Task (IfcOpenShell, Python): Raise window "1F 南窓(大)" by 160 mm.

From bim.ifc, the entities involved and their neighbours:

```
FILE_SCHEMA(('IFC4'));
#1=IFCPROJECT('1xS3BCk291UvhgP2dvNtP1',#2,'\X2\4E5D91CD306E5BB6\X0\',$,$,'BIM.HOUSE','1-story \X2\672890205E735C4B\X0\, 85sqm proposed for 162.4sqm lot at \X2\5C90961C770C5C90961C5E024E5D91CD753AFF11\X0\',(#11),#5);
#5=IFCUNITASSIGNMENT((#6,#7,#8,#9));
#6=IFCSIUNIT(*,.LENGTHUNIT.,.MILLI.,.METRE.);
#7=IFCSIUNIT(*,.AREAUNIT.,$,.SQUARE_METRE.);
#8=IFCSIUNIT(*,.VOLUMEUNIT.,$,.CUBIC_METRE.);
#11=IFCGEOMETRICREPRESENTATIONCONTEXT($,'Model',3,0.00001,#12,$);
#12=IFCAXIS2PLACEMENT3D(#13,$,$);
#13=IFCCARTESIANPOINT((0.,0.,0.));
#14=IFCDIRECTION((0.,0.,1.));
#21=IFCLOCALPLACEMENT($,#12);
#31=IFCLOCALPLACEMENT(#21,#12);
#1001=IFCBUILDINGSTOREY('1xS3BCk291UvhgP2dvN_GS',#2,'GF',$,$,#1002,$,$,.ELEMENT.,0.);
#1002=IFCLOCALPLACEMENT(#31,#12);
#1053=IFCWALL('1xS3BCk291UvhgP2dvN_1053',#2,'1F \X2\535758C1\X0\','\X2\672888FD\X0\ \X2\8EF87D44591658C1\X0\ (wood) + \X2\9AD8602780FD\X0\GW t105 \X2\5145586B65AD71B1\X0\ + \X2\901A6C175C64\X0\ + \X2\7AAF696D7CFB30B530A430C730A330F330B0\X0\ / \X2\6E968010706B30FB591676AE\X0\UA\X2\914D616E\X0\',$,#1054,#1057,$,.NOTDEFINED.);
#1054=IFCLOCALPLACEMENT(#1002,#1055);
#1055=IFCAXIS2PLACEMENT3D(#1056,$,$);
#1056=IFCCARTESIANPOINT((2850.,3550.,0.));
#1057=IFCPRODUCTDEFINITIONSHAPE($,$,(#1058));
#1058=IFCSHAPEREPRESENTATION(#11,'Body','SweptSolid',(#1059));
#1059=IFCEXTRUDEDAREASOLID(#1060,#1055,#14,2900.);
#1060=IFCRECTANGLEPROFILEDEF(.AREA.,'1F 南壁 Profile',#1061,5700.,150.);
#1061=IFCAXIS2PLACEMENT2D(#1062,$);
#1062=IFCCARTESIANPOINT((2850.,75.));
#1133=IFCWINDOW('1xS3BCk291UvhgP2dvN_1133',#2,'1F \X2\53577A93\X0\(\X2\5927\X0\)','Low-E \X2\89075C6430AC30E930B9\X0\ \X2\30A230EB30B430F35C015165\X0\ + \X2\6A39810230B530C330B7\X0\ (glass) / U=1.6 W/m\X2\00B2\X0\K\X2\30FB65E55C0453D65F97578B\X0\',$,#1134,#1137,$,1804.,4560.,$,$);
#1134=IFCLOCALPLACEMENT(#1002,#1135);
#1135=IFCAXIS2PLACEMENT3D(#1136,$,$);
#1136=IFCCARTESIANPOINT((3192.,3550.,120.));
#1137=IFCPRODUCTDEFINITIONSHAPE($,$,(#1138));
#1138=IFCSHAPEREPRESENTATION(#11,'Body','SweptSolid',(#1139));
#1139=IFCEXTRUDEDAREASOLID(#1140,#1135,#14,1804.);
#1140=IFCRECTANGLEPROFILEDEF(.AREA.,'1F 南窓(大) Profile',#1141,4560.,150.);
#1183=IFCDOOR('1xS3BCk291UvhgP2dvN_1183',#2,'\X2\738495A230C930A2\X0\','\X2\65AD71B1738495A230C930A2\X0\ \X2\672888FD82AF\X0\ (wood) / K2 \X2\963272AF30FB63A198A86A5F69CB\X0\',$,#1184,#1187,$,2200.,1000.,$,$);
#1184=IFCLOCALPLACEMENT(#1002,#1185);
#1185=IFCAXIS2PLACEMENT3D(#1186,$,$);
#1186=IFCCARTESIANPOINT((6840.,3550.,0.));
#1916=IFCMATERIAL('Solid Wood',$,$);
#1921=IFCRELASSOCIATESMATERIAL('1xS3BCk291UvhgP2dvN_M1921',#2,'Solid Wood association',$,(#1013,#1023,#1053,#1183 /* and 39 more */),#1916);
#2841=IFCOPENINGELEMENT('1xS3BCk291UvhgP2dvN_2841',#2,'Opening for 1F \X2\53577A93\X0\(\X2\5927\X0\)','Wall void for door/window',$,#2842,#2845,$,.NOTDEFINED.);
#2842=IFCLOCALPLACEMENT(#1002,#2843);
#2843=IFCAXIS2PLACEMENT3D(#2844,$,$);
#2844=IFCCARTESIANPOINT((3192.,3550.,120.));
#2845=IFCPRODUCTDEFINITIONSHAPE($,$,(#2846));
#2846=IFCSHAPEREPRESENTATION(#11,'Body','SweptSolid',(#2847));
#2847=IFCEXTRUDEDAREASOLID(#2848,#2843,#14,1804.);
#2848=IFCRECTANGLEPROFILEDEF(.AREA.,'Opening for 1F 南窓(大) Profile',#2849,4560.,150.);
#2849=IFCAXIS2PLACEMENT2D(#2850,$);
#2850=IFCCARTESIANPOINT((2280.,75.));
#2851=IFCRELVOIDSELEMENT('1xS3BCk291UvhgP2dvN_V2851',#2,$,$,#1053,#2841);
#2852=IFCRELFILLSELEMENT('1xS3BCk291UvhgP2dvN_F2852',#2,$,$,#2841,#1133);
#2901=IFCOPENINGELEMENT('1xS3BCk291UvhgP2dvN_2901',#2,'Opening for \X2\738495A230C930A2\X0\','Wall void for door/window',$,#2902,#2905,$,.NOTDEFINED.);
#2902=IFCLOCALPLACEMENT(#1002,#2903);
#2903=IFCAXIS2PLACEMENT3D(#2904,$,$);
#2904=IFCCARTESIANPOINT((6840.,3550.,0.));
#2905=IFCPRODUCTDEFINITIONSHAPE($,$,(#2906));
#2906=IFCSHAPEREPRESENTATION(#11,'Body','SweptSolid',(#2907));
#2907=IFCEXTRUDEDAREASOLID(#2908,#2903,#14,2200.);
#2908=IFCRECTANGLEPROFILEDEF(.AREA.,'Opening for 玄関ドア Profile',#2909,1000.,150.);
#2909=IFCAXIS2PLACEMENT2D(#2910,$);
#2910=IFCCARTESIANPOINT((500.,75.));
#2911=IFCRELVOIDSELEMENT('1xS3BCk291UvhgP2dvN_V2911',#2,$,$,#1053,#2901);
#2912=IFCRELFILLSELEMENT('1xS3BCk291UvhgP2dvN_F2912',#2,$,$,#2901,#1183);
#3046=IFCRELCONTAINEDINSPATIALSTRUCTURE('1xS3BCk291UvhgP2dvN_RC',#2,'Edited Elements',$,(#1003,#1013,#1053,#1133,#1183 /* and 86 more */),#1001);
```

```python
import numpy as np
import ifcopenshell
import ifcopenshell.api.geometry
import ifcopenshell.util.placement
import ifcopenshell.util.unit

model = ifcopenshell.open("bim.ifc")
unit_scale = ifcopenshell.util.unit.calculate_unit_scale(model)

window = model.by_guid("1xS3BCk291UvhgP2dvN_1133")
opening = window.FillsVoids[0].RelatingOpeningElement
dz = 160.0

shift = np.array([0.0, 0.0, dz])
# The window is not placed relative to its opening, so move both.
for product in (opening, window):
    matrix = ifcopenshell.util.placement.get_local_placement(product.ObjectPlacement)
    matrix[:3, 3] += shift
    ifcopenshell.api.geometry.edit_object_placement(model, product=product, matrix=matrix, is_si=False)

print(f"moved by {dz * unit_scale:+.3f} m")

model.write("bim_v2.ifc")
```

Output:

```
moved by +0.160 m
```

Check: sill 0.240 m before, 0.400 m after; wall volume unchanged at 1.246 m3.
